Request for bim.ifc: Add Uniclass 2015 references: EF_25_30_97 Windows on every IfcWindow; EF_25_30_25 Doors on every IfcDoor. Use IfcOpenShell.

First a look at what the model holds.

```python
import ifcopenshell

model = ifcopenshell.open("bim.ifc")
print(model.schema)
print("classifications:", [c.Name for c in model.by_type("IfcClassification")])
for ifc_class in ("IfcDoor", "IfcRoof", "IfcStair", "IfcWall", "IfcWindow"):
    print(ifc_class, len(model.by_type(ifc_class)))
```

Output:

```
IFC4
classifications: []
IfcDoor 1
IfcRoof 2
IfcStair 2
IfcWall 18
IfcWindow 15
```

```python
import ifcopenshell
import ifcopenshell.api.classification

model = ifcopenshell.open("bim.ifc")

system = ifcopenshell.api.classification.add_classification(model, classification="Uniclass 2015")

codes = {
    "IfcWindow": ("EF_25_30_97", "Windows"),
    "IfcDoor": ("EF_25_30_25", "Doors"),
}
for ifc_class, (code, name) in codes.items():
    products = model.by_type(ifc_class)
    ifcopenshell.api.classification.add_reference(
        model, products=products, classification=system, identification=code, name=name
    )
    print(code, len(products))

model.write("bim_edited.ifc")
```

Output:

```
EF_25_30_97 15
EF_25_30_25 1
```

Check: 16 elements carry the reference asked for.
